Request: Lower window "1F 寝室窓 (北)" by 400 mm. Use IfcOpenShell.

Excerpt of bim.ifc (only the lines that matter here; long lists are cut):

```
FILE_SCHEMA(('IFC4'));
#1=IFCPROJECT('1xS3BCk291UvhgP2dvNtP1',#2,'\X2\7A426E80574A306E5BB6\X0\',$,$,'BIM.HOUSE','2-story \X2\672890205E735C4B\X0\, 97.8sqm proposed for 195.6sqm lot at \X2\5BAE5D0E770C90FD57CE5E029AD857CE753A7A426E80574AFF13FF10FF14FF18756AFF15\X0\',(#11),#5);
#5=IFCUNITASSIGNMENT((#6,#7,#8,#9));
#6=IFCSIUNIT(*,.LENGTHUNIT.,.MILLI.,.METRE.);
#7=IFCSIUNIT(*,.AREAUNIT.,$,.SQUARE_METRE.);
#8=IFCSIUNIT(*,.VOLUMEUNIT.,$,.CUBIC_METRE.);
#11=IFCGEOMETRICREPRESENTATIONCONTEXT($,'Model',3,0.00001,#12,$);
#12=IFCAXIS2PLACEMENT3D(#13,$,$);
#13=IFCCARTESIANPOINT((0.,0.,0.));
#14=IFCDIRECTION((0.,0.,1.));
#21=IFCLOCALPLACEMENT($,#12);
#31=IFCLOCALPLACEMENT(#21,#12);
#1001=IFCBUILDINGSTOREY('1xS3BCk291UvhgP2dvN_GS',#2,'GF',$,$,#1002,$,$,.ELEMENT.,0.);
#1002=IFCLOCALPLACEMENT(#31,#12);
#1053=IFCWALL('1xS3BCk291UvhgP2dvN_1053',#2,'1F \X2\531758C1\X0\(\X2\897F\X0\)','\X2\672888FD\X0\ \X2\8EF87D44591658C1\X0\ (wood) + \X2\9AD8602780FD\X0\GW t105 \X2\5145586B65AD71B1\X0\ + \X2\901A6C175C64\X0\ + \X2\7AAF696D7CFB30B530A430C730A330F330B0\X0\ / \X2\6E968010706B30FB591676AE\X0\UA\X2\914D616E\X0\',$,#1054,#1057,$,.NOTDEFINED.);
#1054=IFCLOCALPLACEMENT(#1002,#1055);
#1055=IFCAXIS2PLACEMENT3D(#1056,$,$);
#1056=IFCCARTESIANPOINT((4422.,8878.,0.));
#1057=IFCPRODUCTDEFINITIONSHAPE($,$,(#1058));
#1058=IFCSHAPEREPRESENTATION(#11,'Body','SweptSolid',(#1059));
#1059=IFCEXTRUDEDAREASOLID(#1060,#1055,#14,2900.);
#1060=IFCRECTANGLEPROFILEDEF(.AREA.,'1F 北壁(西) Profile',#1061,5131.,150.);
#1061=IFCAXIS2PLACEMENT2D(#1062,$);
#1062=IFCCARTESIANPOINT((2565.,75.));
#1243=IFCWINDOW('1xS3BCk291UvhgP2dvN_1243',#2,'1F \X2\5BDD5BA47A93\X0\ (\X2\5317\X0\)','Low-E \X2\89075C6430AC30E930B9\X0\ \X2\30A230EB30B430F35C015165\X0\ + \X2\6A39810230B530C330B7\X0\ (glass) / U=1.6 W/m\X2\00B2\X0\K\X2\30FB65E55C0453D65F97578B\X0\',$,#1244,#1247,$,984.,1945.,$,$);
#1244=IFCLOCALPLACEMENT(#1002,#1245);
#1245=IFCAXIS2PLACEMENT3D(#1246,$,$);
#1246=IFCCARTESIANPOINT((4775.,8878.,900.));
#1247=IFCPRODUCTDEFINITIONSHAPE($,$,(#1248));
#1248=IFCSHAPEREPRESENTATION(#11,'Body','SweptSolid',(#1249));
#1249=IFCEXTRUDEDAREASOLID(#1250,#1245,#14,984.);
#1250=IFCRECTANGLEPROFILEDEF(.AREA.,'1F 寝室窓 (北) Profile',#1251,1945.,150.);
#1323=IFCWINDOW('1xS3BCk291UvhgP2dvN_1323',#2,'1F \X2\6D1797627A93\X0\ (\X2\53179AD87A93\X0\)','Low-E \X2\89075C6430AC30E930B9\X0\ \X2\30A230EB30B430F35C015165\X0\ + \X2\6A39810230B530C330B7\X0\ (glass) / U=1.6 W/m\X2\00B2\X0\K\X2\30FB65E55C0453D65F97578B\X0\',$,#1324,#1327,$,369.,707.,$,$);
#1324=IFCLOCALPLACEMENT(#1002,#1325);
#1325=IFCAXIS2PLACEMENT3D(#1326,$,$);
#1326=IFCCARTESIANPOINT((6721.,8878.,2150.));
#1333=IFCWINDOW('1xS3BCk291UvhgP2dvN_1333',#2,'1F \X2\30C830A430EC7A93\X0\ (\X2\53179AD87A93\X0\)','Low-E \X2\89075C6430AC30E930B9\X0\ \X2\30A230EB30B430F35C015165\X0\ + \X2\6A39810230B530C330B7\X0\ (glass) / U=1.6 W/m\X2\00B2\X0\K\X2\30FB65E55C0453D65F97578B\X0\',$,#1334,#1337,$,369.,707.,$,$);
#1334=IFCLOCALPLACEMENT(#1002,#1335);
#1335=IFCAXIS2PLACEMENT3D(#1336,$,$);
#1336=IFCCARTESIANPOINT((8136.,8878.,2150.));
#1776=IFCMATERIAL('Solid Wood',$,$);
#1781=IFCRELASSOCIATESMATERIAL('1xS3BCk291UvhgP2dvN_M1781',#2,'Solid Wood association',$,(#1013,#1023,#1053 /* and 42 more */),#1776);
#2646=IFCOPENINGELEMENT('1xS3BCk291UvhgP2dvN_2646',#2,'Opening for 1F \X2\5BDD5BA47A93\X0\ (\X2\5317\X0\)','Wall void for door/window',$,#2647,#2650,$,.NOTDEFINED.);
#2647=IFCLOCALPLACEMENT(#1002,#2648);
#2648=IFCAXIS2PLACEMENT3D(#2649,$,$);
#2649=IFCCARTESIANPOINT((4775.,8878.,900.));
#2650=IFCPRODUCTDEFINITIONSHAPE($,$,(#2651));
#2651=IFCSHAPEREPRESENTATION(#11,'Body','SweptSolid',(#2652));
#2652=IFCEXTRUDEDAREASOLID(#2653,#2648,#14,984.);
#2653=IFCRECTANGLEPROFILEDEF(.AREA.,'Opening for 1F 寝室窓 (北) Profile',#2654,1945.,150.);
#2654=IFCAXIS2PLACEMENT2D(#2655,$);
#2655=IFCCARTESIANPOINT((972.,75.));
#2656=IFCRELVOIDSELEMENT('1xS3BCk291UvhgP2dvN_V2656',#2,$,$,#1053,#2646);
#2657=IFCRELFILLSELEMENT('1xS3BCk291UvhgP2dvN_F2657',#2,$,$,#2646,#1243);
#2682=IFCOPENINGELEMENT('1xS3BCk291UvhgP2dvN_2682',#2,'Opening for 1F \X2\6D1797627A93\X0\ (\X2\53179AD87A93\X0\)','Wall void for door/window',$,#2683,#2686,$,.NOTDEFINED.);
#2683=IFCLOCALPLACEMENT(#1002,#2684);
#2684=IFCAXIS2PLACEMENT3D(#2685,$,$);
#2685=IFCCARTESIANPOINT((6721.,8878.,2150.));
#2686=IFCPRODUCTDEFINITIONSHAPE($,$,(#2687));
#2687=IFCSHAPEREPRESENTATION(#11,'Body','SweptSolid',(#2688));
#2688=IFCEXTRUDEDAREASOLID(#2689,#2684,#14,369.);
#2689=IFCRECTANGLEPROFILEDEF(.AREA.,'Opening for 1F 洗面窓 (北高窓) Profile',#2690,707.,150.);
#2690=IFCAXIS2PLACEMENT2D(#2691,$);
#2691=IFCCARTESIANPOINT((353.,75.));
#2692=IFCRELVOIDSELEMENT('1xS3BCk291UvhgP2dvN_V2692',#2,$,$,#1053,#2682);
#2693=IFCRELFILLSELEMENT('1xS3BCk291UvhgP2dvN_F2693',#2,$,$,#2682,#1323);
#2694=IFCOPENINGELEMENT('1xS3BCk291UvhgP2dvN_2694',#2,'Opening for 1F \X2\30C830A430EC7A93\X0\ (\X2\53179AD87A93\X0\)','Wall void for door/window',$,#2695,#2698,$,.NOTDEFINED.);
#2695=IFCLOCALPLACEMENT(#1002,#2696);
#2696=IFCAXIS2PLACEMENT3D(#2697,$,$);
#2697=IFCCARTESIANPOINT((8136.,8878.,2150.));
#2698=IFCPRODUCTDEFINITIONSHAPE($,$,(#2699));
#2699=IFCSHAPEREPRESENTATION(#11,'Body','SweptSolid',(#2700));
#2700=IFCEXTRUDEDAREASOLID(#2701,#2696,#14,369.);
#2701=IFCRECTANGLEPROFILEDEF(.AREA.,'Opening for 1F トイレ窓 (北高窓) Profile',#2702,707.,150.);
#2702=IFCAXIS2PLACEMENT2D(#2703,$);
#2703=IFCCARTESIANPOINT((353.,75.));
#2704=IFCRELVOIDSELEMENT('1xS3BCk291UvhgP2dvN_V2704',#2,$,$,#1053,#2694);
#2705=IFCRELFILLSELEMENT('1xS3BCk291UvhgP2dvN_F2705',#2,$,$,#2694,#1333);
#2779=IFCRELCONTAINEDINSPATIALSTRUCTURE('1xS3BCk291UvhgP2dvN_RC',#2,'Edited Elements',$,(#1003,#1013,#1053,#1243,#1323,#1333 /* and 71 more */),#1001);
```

```python
import numpy as np
import ifcopenshell
import ifcopenshell.api.geometry
import ifcopenshell.util.placement
import ifcopenshell.util.unit

model = ifcopenshell.open("bim.ifc")
unit_scale = ifcopenshell.util.unit.calculate_unit_scale(model)

window = model.by_id(1243)
opening = window.FillsVoids[0].RelatingOpeningElement
dz = -0.4 / unit_scale

shift = np.array([0.0, 0.0, dz])
# The window is not placed relative to its opening, so move both.
for product in (opening, window):
    matrix = ifcopenshell.util.placement.get_local_placement(product.ObjectPlacement)
    matrix[:3, 3] += shift
    ifcopenshell.api.geometry.edit_object_placement(model, product=product, matrix=matrix, is_si=False)

print(f"moved by {dz * unit_scale:+.3f} m")

model.write("bim_updated.ifc")
```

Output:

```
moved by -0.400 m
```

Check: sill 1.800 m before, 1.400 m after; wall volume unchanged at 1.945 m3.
